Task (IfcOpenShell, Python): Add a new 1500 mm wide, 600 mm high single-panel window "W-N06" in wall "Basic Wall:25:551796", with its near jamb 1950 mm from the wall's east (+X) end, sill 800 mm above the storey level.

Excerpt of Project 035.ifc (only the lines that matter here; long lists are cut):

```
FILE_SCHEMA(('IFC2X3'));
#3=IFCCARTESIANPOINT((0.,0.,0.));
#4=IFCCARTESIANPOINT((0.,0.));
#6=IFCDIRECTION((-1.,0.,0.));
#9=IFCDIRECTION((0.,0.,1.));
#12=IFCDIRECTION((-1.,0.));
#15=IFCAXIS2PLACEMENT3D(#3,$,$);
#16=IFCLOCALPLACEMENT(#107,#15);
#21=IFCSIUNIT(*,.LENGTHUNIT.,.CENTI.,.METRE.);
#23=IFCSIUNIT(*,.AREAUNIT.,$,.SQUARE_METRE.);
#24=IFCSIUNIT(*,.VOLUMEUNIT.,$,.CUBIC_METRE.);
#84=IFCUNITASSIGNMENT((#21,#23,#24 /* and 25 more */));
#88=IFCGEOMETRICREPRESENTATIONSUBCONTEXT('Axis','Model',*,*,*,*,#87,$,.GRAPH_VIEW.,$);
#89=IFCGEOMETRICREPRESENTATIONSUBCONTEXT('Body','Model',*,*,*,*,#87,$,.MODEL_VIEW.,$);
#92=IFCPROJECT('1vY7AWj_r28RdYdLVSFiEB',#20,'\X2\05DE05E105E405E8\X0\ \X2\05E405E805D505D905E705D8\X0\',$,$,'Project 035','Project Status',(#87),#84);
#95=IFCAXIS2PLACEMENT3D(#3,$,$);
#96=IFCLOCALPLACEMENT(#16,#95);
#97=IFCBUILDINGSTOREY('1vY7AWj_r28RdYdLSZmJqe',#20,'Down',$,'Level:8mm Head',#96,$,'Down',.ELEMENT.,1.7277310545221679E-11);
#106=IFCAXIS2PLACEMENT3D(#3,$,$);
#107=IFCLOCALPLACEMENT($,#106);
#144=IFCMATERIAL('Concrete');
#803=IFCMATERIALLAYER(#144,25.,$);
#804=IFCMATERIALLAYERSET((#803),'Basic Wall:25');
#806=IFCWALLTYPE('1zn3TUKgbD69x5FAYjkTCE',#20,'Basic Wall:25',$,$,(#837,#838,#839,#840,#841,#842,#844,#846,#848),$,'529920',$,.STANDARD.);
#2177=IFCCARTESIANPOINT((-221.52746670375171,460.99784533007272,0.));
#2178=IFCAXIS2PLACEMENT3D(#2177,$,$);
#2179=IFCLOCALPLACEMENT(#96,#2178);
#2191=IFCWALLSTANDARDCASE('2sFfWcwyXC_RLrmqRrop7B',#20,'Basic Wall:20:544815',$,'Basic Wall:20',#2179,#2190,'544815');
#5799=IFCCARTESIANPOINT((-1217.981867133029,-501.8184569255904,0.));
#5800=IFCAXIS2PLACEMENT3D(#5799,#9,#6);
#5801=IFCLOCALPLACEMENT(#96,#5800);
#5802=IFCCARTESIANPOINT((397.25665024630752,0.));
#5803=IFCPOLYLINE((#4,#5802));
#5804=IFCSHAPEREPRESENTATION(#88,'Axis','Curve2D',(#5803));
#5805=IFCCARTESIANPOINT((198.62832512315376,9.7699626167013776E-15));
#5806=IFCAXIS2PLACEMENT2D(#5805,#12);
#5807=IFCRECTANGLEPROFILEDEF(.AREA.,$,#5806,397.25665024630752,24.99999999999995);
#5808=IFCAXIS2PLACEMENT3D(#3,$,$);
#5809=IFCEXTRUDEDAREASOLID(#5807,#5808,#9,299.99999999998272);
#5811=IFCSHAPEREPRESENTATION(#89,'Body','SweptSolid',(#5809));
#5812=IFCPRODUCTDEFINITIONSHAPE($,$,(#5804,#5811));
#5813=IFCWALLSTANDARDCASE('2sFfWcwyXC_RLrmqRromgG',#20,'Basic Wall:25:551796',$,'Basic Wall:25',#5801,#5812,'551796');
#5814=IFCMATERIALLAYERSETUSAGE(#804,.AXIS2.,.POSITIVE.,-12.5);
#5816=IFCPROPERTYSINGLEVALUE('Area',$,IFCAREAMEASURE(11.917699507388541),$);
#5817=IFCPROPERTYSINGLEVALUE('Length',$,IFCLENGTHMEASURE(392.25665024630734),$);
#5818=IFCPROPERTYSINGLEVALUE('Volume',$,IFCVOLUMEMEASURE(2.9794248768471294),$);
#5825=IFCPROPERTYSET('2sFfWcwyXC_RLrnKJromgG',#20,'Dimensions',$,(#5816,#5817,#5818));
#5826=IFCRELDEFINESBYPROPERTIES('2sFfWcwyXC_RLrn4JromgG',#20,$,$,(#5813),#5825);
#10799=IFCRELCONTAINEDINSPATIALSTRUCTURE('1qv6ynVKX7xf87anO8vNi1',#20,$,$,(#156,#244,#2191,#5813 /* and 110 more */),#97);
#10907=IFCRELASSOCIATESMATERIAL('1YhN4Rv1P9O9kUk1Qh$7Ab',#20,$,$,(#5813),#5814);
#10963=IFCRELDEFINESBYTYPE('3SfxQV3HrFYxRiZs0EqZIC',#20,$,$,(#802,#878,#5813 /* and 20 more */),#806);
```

```python
import numpy as np
import ifcopenshell
import ifcopenshell.api.feature
import ifcopenshell.api.geometry
import ifcopenshell.api.pset
import ifcopenshell.api.root
import ifcopenshell.api.spatial
import ifcopenshell.api.type
import ifcopenshell.geom
import ifcopenshell.util.element
import ifcopenshell.util.placement
import ifcopenshell.util.representation
import ifcopenshell.util.shape
import ifcopenshell.util.unit

model = ifcopenshell.open("Project 035.ifc")
unit_scale = ifcopenshell.util.unit.calculate_unit_scale(model)
area_scale = ifcopenshell.util.unit.calculate_unit_scale(model, "AREAUNIT")
volume_scale = ifcopenshell.util.unit.calculate_unit_scale(model, "VOLUMEUNIT")
settings = ifcopenshell.geom.settings()


def volume(element):
    """Net volume in cubic metres, openings subtracted."""
    shape = ifcopenshell.geom.create_shape(settings, element)
    return ifcopenshell.util.shape.get_volume(shape.geometry)


wall = model.by_id(5813)
storey = ifcopenshell.util.element.get_container(wall, ifc_class="IfcBuildingStorey")
context = ifcopenshell.util.representation.get_context(model, "Model", "Body", "MODEL_VIEW")
before = volume(wall)

width, height, from_end, sill = 1.5, 0.6, 1.95, 0.8  # metres

# The wall runs along its own X axis, and the end named is its -X end.
wall_shape = ifcopenshell.geom.create_shape(settings, wall)
x, y, z = ifcopenshell.util.shape.get_vertices(wall_shape.geometry).T
start = x.min() + from_end
face, thickness = float(y.min()), float(y.max() - y.min())
wall_matrix = ifcopenshell.util.placement.get_local_placement(wall.ObjectPlacement)
level = ifcopenshell.util.placement.get_local_placement(storey.ObjectPlacement)[2, 3]


def in_wall(x, y):
    """Placement at x, y metres in the wall's axes, at sill height."""
    matrix = wall_matrix.copy()
    matrix[:, 3] = wall_matrix @ np.array([x / unit_scale, y / unit_scale, 0.0, 1.0])
    matrix[2, 3] = level + sill / unit_scale
    return matrix


# Opening: a box that overshoots both wall faces by 50 mm.
opening = ifcopenshell.api.root.create_entity(model, ifc_class="IfcOpeningElement")
box = ifcopenshell.api.geometry.add_wall_representation(
    model, context=context, length=width, height=height, thickness=thickness + 0.1
)
ifcopenshell.api.geometry.assign_representation(model, product=opening, representation=box)
ifcopenshell.api.geometry.edit_object_placement(model, product=opening, matrix=in_wall(start, face - 0.05), is_si=False)
ifcopenshell.api.feature.add_feature(model, feature=opening, element=wall)

window = ifcopenshell.api.root.create_entity(model, ifc_class="IfcWindow", name="W-N06")
window.OverallWidth, window.OverallHeight = width / unit_scale, height / unit_scale
body = ifcopenshell.api.geometry.add_window_representation(
    model,
    context=context,
    overall_width=window.OverallWidth,
    overall_height=window.OverallHeight,
    partition_type="SINGLE_PANEL",
)
ifcopenshell.api.geometry.assign_representation(model, product=window, representation=body)
ifcopenshell.api.spatial.assign_container(model, products=[window], relating_structure=storey)
fills = ifcopenshell.api.feature.add_filling(model, opening=opening, element=window)
fills.OwnerHistory = window.OwnerHistory  # required in IFC2X3

# IFC2X3 keeps the operation on the window style.
style = ifcopenshell.api.root.create_entity(model, ifc_class="IfcWindowStyle", name="W-N06")
style.OperationType, style.ConstructionType = "SINGLE_PANEL", "NOTDEFINED"
style.ParameterTakesPrecedence = style.Sizeable = False
ifcopenshell.api.type.assign_type(model, related_objects=[window], relating_type=style)

# Centre the window in the wall's thickness.
ifcopenshell.api.geometry.edit_object_placement(model, product=window, matrix=in_wall(start, face), is_si=False)
window_shape = ifcopenshell.geom.create_shape(settings, window)
depth = ifcopenshell.util.shape.get_vertices(window_shape.geometry)[:, 1]
offset = face + thickness / 2 - (depth.min() + depth.max()) / 2
ifcopenshell.api.geometry.edit_object_placement(model, product=window, matrix=in_wall(start, offset), is_si=False)

after = volume(wall)

# Update the wall's stored quantities.
pset = model.by_id(ifcopenshell.util.element.get_pset(wall, "Dimensions", should_inherit=False)["id"])
ifcopenshell.api.pset.edit_pset(model, pset=pset, properties={
    "Area": model.create_entity("IfcAreaMeasure", after / thickness / area_scale),
    "Volume": model.create_entity("IfcVolumeMeasure", after / volume_scale),
})

print(f"wall volume {before:.3f} -> {after:.3f} m3")

model.write("Project 035_rev.ifc")
```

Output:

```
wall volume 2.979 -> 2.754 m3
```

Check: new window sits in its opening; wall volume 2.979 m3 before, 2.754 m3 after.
